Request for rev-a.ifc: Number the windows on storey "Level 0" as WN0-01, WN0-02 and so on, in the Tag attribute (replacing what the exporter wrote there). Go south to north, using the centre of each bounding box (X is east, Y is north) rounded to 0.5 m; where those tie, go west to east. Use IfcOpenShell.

First a look at what the model holds.

```python
import ifcopenshell
import ifcopenshell.util.element
import ifcopenshell.util.placement

model = ifcopenshell.open("rev-a.ifc")
print(model.schema)
storey = next(s for s in model.by_type("IfcBuildingStorey") if s.Name == "Level 0")
windows = [e for e in ifcopenshell.util.element.get_decomposition(storey) if e.is_a("IfcWindow")]
for e in sorted(windows, key=lambda e: e.id()):
    origin = ifcopenshell.util.placement.get_local_placement(e.ObjectPlacement)[:3, 3]
    print(e.id(), e.Tag, e.Name, origin.round(2) + 0.0, sep=" | ")
```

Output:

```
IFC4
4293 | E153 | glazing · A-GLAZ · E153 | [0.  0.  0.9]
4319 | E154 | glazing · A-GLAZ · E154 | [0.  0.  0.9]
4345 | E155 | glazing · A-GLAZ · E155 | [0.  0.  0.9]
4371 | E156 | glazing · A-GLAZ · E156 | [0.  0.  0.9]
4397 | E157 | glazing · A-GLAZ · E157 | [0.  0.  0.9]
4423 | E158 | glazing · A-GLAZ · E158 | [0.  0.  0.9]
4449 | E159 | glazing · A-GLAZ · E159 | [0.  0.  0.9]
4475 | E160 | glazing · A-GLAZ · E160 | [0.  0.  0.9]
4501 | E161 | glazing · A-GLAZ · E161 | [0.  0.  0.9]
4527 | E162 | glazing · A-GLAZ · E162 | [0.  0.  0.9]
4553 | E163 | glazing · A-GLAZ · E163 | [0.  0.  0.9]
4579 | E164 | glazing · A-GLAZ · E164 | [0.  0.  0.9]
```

```python
import ifcopenshell
import ifcopenshell.geom
import ifcopenshell.util.element
import ifcopenshell.util.shape

model = ifcopenshell.open("rev-a.ifc")
settings = ifcopenshell.geom.settings()
settings.set("use-world-coords", True)


def centre(element):
    shape = ifcopenshell.geom.create_shape(settings, element)
    return ifcopenshell.util.shape.get_bbox_centroid(shape.geometry)


storey = next(s for s in model.by_type("IfcBuildingStorey") if s.Name == "Level 0")
windows = [e for e in ifcopenshell.util.element.get_decomposition(storey) if e.is_a("IfcWindow")]

# Insertion points can sit at a corner or the storey origin, so sort by the geometry (in metres).
centres = {e: centre(e) for e in windows}
windows.sort(key=lambda e: (round(centres[e][1] / 0.5), centres[e][0]))

for i, e in enumerate(windows, start=1):
    number = f"WN0-{i:02d}"
    e.Tag = number
    print(e.id(), number)

model.write("rev-a_edited.ifc")
```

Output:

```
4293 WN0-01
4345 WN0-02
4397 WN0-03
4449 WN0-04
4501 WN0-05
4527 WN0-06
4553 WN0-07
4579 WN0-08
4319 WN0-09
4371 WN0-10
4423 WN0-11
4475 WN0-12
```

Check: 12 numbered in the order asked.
